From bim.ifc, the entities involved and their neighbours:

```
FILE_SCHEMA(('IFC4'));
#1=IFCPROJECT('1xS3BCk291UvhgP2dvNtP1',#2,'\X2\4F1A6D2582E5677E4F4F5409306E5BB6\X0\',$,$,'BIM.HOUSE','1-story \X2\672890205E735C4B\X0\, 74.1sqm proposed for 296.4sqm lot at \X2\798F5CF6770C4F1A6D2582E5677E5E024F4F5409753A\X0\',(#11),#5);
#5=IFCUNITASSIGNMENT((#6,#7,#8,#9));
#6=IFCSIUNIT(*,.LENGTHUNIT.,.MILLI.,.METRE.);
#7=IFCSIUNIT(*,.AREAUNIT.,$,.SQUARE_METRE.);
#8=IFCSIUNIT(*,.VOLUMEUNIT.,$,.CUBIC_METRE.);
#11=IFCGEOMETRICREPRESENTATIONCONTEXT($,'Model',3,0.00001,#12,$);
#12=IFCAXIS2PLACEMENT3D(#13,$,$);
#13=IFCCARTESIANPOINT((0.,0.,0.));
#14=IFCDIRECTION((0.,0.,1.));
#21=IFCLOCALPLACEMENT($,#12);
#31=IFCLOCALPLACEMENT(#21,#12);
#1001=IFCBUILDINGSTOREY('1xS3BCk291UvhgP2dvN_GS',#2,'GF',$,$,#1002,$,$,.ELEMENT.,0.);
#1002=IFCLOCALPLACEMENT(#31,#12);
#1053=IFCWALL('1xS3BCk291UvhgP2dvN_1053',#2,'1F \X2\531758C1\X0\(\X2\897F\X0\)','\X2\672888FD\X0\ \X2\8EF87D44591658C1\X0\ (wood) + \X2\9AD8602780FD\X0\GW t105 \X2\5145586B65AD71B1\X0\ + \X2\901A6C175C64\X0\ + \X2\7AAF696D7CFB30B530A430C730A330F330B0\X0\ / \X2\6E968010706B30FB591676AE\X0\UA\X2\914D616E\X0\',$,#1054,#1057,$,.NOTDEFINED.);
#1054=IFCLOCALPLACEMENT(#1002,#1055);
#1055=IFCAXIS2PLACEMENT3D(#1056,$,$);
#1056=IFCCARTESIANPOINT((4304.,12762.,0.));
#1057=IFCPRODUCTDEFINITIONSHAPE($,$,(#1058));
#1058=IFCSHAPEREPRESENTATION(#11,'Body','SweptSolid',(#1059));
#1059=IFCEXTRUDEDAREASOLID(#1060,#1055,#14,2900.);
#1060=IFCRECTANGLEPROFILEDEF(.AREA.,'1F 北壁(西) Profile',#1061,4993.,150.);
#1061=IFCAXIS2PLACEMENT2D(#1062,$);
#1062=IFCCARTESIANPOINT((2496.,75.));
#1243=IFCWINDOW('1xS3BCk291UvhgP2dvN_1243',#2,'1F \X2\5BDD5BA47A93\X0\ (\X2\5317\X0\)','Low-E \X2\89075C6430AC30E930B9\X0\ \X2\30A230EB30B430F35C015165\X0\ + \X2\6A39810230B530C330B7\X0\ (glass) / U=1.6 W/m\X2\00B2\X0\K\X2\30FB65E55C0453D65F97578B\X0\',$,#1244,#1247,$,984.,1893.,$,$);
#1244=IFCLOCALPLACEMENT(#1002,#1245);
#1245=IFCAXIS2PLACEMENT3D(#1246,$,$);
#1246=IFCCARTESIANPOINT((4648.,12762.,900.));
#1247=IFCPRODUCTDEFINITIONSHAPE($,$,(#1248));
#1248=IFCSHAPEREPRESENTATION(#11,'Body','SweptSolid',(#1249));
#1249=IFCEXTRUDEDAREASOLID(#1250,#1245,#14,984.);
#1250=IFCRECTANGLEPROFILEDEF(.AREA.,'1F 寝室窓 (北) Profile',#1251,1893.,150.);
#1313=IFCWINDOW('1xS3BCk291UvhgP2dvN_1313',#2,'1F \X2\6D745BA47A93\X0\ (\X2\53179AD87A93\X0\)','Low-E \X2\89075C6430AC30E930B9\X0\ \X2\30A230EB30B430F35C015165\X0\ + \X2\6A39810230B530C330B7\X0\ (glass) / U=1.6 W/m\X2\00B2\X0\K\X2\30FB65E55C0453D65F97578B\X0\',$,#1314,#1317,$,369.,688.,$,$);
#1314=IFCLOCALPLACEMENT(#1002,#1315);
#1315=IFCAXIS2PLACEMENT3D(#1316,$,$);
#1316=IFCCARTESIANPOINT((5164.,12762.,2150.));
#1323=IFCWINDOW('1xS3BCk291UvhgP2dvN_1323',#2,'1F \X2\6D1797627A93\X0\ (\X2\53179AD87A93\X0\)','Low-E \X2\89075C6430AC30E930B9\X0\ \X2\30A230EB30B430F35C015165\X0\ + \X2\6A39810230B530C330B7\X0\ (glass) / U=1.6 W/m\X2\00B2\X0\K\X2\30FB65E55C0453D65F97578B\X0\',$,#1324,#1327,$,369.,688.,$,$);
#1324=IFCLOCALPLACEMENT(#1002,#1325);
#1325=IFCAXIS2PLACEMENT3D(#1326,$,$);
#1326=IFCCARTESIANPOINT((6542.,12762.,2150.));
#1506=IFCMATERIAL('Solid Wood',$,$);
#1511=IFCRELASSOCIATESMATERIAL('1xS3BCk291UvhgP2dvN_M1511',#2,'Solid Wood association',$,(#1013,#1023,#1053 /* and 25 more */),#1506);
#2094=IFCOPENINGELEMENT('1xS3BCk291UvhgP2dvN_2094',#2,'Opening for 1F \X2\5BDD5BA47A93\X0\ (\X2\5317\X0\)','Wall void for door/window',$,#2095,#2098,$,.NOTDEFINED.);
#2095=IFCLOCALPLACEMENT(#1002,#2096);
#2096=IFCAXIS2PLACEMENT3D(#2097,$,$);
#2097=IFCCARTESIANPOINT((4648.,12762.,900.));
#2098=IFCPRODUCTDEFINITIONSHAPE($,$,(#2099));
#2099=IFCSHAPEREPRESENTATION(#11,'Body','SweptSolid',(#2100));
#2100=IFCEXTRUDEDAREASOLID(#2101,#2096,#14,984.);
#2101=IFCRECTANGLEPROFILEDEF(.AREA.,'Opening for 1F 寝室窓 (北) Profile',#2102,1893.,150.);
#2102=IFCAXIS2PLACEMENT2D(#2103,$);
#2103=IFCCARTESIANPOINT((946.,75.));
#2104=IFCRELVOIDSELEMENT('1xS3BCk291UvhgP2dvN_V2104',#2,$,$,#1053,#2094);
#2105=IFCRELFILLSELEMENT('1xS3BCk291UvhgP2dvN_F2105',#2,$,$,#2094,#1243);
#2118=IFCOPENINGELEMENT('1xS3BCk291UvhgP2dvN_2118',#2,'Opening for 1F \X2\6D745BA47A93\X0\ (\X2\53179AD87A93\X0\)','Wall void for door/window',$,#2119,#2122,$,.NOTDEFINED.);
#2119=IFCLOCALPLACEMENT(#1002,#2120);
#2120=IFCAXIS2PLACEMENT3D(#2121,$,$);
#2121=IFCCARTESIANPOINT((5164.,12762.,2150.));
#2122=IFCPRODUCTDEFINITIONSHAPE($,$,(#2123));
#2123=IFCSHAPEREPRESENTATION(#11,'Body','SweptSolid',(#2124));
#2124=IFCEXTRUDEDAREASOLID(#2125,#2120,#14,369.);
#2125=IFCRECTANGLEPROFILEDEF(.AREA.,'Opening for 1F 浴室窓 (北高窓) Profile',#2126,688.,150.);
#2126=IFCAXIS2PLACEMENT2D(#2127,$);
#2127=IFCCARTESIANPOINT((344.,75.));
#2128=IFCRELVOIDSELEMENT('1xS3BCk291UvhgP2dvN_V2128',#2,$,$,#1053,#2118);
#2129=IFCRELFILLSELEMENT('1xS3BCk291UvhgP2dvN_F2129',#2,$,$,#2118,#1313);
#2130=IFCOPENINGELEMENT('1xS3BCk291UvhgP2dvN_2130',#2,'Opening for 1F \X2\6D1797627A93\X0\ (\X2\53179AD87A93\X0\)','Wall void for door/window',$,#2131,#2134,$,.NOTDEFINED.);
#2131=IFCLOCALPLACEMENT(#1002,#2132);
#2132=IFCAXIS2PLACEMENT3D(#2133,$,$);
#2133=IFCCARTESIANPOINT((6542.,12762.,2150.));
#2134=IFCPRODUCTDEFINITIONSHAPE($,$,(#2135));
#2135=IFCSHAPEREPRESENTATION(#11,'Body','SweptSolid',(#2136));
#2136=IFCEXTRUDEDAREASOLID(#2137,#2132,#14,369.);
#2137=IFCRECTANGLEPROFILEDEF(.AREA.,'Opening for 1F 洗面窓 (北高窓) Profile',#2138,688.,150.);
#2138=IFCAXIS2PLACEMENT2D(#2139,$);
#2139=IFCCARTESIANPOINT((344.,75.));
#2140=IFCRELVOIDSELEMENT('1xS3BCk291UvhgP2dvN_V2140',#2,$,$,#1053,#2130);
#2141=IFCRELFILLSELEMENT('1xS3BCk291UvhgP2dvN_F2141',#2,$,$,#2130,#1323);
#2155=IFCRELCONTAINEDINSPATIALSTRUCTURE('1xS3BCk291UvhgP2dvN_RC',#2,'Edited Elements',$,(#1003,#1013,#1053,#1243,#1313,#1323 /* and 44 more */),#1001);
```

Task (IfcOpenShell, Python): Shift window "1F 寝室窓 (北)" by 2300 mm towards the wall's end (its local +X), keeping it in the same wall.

```python
import ifcopenshell
import ifcopenshell.api.geometry
import ifcopenshell.util.placement

model = ifcopenshell.open("bim.ifc")

window = model.by_guid("1xS3BCk291UvhgP2dvN_1243")
opening = window.FillsVoids[0].RelatingOpeningElement
wall = opening.VoidsElements[0].RelatingBuildingElement

wall_matrix = ifcopenshell.util.placement.get_local_placement(wall.ObjectPlacement)
shift = wall_matrix[:3, 0] * 2300.0
before = ifcopenshell.util.placement.get_local_placement(window.ObjectPlacement)[:3, 3].copy()

# The window is not placed relative to its opening, so move both.
for product in (opening, window):
    matrix = ifcopenshell.util.placement.get_local_placement(product.ObjectPlacement)
    matrix[:3, 3] += shift
    ifcopenshell.api.geometry.edit_object_placement(model, product=product, matrix=matrix, is_si=False)

after = ifcopenshell.util.placement.get_local_placement(window.ObjectPlacement)[:3, 3]
print("window moved by", (after - before).round(3) + 0.0)

model.write("bim-out.ifc")
```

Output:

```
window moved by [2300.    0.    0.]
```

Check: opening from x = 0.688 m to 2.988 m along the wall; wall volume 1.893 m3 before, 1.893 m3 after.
